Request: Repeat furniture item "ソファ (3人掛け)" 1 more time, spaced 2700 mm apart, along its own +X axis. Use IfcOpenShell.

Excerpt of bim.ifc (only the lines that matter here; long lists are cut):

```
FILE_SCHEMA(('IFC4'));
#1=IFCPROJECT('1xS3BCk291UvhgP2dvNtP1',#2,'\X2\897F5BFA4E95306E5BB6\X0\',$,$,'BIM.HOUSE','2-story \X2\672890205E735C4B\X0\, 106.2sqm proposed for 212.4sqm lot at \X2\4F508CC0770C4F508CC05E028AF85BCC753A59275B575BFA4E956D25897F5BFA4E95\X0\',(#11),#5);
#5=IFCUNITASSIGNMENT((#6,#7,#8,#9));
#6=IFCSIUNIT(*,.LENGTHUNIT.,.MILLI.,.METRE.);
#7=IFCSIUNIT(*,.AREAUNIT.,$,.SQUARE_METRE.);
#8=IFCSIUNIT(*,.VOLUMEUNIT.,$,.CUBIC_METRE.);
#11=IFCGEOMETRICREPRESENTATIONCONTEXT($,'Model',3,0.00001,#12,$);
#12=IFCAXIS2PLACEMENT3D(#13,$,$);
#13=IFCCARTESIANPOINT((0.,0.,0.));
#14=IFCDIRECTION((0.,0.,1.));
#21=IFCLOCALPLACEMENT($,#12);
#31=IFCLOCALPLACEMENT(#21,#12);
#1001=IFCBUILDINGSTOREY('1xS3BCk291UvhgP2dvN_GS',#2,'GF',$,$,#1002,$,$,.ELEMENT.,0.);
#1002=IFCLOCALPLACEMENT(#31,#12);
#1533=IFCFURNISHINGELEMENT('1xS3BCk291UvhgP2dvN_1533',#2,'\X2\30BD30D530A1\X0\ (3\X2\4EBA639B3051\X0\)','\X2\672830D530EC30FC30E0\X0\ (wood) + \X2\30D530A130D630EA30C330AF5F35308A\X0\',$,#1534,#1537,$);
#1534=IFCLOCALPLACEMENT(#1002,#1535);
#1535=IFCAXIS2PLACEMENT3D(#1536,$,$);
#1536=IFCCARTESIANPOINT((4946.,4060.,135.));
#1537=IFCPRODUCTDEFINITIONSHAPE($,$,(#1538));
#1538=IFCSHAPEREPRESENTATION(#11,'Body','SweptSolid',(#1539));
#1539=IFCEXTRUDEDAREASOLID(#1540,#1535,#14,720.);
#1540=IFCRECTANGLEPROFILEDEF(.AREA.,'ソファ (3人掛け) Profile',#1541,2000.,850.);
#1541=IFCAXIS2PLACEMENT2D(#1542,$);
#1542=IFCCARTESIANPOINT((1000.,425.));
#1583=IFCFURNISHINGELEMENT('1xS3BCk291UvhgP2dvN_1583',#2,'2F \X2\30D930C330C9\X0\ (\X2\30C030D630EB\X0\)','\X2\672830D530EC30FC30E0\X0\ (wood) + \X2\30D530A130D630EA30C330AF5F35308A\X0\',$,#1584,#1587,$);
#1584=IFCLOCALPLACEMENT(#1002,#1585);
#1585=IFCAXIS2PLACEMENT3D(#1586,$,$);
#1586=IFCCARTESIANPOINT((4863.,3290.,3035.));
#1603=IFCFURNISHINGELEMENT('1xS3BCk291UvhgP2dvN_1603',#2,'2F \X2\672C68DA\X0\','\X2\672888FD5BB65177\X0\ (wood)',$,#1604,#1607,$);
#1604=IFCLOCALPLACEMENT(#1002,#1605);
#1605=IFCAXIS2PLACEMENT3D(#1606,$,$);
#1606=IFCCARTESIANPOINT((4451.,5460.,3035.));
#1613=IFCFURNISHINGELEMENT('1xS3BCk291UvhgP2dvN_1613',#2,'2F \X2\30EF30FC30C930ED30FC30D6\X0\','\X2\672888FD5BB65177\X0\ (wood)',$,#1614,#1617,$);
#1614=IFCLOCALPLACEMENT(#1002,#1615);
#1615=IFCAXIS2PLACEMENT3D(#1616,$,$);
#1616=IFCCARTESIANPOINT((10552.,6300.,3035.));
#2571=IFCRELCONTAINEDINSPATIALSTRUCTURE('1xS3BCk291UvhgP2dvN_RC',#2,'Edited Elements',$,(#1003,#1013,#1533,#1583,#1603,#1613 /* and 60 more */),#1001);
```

```python
import ifcopenshell
import ifcopenshell.api.geometry
import ifcopenshell.api.root
import ifcopenshell.util.element
import ifcopenshell.util.placement

model = ifcopenshell.open("bim.ifc")


def reuse_history(source, copy):
    """copy_class also copies each property set's owner history, people and application; keep the originals."""
    for rel in copy.IsDefinedBy:
        if rel.is_a("IfcRelDefinesByProperties") and (history := rel.RelatingPropertyDefinition.OwnerHistory):
            rel.RelatingPropertyDefinition.OwnerHistory = source.OwnerHistory
            ifcopenshell.util.element.remove_deep2(model, history)


source = model.by_guid("1xS3BCk291UvhgP2dvN_1533")
base = ifcopenshell.util.placement.get_local_placement(source.ObjectPlacement)
step = base[:3, 0] * 2700.0

for i in range(1, 2):
    copy = ifcopenshell.api.root.copy_class(model, product=source)
    copy.Representation = ifcopenshell.util.element.copy_deep(
        model, source.Representation, exclude=["IfcGeometricRepresentationContext", "IfcRepresentationMap"]
    )
    reuse_history(source, copy)
    matrix = base.copy()
    matrix[:3, 3] += i * step
    print("added at", matrix[:3, 3].round(3) + 0.0)
    ifcopenshell.api.geometry.edit_object_placement(model, product=copy, matrix=matrix, is_si=False)

model.write("bim-out.ifc")
```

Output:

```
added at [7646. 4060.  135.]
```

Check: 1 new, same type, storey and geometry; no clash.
